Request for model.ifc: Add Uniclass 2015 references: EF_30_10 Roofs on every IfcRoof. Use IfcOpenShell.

First a look at what the model holds.

```python
import ifcopenshell

model = ifcopenshell.open("model.ifc")
print(model.schema)
print("classifications:", [c.Name for c in model.by_type("IfcClassification")])
for ifc_class in ("IfcDoor", "IfcRoof", "IfcStair", "IfcWall", "IfcWindow"):
    print(ifc_class, len(model.by_type(ifc_class)))
```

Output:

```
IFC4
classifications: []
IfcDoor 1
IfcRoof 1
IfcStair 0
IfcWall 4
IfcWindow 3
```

```python
import ifcopenshell
import ifcopenshell.api.classification

model = ifcopenshell.open("model.ifc")

system = ifcopenshell.api.classification.add_classification(model, classification="Uniclass 2015")

codes = {
    "IfcRoof": ("EF_30_10", "Roofs"),
}
for ifc_class, (code, name) in codes.items():
    products = model.by_type(ifc_class)
    ifcopenshell.api.classification.add_reference(
        model, products=products, classification=system, identification=code, name=name
    )
    print(code, len(products))

model.write("model-out.ifc")
```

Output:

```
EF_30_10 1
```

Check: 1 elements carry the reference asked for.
